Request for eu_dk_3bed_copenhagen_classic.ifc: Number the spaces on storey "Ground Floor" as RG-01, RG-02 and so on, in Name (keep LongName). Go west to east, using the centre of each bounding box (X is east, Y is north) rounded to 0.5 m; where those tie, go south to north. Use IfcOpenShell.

First a look at what the model holds.

```python
import ifcopenshell
import ifcopenshell.util.element
import ifcopenshell.util.placement

model = ifcopenshell.open("eu_dk_3bed_copenhagen_classic.ifc")
print(model.schema)
storey = next(s for s in model.by_type("IfcBuildingStorey") if s.Name == "Ground Floor")
spaces = [e for e in ifcopenshell.util.element.get_decomposition(storey) if e.is_a("IfcSpace")]
for e in sorted(spaces, key=lambda e: e.id()):
    origin = ifcopenshell.util.placement.get_local_placement(e.ObjectPlacement)[:3, 3]
    print(e.id(), e.Name, e.LongName, origin.round(2) + 0.0, sep=" | ")
```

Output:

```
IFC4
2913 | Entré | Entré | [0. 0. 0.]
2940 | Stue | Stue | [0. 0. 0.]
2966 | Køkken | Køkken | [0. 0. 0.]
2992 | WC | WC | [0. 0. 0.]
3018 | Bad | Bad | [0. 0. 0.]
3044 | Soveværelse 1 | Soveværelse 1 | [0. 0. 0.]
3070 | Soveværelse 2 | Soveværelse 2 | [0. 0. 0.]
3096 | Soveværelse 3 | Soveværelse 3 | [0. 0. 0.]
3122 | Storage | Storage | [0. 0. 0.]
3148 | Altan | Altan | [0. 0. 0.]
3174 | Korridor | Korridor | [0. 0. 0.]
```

```python
import ifcopenshell
import ifcopenshell.geom
import ifcopenshell.util.element
import ifcopenshell.util.shape

model = ifcopenshell.open("eu_dk_3bed_copenhagen_classic.ifc")
settings = ifcopenshell.geom.settings()
settings.set("use-world-coords", True)


def centre(element):
    shape = ifcopenshell.geom.create_shape(settings, element)
    return ifcopenshell.util.shape.get_bbox_centroid(shape.geometry)


storey = next(s for s in model.by_type("IfcBuildingStorey") if s.Name == "Ground Floor")
spaces = [e for e in ifcopenshell.util.element.get_decomposition(storey) if e.is_a("IfcSpace")]

# Insertion points can sit at a corner or the storey origin, so sort by the geometry (in metres).
centres = {e: centre(e) for e in spaces}
spaces.sort(key=lambda e: (round(centres[e][0] / 0.5), centres[e][1]))

for i, e in enumerate(spaces, start=1):
    number = f"RG-{i:02d}"
    e.Name = number
    print(e.id(), number)

model.write("eu_dk_3bed_copenhagen_classic_rev.ifc")
```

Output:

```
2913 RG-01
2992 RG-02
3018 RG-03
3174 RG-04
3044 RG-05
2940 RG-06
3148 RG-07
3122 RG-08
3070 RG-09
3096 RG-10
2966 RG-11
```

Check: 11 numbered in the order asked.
